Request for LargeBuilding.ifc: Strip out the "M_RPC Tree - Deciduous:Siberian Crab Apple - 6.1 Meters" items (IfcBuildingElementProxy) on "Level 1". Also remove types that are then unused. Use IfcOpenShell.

First a look at what the model holds.

```python
import ifcopenshell
import ifcopenshell.util.element

model = ifcopenshell.open("LargeBuilding.ifc")
print(model.schema)
storey = next(s for s in model.by_type("IfcBuildingStorey") if s.Name == "Level 1")
proxies = [e for e in ifcopenshell.util.element.get_decomposition(storey) if e.is_a("IfcBuildingElementProxy")]
seen = {}
for e in proxies:
    element_type = ifcopenshell.util.element.get_type(e)
    name = element_type.Name if element_type not in (None, e) else None
    seen[name] = seen.get(name, 0) + 1
for name, count in sorted(seen.items(), key=str):
    print(count, "x", name)
```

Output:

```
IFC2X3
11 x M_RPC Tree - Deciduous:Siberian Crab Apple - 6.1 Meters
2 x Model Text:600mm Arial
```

```python
import ifcopenshell
import ifcopenshell.api.root
import ifcopenshell.util.element

model = ifcopenshell.open("LargeBuilding.ifc")

storey = next(s for s in model.by_type("IfcBuildingStorey") if s.Name == "Level 1")
proxies = [e for e in ifcopenshell.util.element.get_decomposition(storey) if e.is_a("IfcBuildingElementProxy")]
targets = [e for e in proxies if (t := ifcopenshell.util.element.get_type(e)) not in (None, e) and t.Name == "M_RPC Tree - Deciduous:Siberian Crab Apple - 6.1 Meters"]
types = {ifcopenshell.util.element.get_type(e) for e in targets} - {None, *targets}

for e in targets:
    ifcopenshell.api.root.remove_product(model, product=e)
print(len(targets), "removed")

unused = [t for t in types if not ifcopenshell.util.element.get_types(t)]
for t in unused:
    ifcopenshell.api.root.remove_product(model, product=t)
print(len(unused), "unused types removed")

model.write("LargeBuilding-out.ifc")
```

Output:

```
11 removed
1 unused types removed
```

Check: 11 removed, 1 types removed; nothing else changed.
